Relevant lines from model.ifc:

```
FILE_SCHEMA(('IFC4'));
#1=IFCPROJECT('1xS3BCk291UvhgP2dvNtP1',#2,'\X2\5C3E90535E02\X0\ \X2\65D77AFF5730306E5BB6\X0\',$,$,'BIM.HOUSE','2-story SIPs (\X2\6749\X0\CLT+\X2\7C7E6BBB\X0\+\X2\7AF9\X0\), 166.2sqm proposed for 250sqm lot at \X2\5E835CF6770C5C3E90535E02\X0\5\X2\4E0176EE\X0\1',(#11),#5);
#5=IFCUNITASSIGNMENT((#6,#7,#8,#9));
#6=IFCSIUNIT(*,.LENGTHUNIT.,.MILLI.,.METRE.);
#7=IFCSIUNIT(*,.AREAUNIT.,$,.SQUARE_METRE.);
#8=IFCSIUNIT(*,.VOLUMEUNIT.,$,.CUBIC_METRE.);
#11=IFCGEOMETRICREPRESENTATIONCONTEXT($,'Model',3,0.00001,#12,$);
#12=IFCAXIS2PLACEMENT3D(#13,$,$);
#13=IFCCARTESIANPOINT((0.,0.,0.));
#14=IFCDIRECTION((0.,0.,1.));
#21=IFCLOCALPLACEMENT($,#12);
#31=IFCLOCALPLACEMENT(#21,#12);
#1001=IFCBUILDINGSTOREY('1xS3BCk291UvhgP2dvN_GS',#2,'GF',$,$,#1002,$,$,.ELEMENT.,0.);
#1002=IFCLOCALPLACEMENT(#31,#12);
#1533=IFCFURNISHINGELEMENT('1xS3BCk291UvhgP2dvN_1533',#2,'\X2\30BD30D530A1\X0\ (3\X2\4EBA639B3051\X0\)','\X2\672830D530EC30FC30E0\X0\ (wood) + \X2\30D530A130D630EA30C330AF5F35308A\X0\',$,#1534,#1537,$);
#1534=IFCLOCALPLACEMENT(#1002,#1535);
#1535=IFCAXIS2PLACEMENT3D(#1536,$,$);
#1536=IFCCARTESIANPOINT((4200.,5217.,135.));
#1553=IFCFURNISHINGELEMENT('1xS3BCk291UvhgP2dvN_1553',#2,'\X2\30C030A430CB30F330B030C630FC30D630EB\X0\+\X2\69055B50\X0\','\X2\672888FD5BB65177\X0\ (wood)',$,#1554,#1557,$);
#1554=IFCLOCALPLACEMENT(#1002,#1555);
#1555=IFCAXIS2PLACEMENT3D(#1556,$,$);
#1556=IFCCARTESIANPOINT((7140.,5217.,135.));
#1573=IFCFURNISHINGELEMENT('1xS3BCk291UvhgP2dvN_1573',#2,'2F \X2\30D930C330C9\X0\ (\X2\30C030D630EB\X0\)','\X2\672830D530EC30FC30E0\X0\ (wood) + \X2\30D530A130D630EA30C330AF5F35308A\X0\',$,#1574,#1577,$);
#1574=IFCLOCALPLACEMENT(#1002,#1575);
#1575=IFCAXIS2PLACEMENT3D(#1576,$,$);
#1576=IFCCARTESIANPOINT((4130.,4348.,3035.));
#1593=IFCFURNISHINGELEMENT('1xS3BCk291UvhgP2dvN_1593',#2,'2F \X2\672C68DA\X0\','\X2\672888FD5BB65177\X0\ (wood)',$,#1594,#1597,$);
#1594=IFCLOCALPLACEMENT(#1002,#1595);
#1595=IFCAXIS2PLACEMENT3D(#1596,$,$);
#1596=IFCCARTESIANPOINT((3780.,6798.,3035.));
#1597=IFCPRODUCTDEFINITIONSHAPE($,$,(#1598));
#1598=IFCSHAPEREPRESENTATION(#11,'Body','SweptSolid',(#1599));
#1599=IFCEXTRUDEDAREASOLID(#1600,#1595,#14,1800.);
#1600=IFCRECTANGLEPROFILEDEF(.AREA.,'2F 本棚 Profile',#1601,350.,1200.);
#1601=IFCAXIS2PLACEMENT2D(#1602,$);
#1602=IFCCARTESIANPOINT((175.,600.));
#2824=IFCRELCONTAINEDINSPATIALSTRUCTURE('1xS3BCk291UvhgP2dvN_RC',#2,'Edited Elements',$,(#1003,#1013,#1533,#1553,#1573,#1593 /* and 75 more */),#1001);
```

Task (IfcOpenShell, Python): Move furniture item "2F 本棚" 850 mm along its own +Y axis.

```python
import ifcopenshell
import ifcopenshell.api.geometry
import ifcopenshell.util.placement
import ifcopenshell.util.unit

model = ifcopenshell.open("model.ifc")
unit_scale = ifcopenshell.util.unit.calculate_unit_scale(model)

item = model.by_id(1593)
matrix = ifcopenshell.util.placement.get_local_placement(item.ObjectPlacement)
matrix[:3, 3] += matrix[:3, 1] * 0.85 / unit_scale
ifcopenshell.api.geometry.edit_object_placement(model, product=item, matrix=matrix, is_si=False)

print(ifcopenshell.util.placement.get_local_placement(item.ObjectPlacement).round(3) + 0.0)

model.write("model_rev.ifc")
```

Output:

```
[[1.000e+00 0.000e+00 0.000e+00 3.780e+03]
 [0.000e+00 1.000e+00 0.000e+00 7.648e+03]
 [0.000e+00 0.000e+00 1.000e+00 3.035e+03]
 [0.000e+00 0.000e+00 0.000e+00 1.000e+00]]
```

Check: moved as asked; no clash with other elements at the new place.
